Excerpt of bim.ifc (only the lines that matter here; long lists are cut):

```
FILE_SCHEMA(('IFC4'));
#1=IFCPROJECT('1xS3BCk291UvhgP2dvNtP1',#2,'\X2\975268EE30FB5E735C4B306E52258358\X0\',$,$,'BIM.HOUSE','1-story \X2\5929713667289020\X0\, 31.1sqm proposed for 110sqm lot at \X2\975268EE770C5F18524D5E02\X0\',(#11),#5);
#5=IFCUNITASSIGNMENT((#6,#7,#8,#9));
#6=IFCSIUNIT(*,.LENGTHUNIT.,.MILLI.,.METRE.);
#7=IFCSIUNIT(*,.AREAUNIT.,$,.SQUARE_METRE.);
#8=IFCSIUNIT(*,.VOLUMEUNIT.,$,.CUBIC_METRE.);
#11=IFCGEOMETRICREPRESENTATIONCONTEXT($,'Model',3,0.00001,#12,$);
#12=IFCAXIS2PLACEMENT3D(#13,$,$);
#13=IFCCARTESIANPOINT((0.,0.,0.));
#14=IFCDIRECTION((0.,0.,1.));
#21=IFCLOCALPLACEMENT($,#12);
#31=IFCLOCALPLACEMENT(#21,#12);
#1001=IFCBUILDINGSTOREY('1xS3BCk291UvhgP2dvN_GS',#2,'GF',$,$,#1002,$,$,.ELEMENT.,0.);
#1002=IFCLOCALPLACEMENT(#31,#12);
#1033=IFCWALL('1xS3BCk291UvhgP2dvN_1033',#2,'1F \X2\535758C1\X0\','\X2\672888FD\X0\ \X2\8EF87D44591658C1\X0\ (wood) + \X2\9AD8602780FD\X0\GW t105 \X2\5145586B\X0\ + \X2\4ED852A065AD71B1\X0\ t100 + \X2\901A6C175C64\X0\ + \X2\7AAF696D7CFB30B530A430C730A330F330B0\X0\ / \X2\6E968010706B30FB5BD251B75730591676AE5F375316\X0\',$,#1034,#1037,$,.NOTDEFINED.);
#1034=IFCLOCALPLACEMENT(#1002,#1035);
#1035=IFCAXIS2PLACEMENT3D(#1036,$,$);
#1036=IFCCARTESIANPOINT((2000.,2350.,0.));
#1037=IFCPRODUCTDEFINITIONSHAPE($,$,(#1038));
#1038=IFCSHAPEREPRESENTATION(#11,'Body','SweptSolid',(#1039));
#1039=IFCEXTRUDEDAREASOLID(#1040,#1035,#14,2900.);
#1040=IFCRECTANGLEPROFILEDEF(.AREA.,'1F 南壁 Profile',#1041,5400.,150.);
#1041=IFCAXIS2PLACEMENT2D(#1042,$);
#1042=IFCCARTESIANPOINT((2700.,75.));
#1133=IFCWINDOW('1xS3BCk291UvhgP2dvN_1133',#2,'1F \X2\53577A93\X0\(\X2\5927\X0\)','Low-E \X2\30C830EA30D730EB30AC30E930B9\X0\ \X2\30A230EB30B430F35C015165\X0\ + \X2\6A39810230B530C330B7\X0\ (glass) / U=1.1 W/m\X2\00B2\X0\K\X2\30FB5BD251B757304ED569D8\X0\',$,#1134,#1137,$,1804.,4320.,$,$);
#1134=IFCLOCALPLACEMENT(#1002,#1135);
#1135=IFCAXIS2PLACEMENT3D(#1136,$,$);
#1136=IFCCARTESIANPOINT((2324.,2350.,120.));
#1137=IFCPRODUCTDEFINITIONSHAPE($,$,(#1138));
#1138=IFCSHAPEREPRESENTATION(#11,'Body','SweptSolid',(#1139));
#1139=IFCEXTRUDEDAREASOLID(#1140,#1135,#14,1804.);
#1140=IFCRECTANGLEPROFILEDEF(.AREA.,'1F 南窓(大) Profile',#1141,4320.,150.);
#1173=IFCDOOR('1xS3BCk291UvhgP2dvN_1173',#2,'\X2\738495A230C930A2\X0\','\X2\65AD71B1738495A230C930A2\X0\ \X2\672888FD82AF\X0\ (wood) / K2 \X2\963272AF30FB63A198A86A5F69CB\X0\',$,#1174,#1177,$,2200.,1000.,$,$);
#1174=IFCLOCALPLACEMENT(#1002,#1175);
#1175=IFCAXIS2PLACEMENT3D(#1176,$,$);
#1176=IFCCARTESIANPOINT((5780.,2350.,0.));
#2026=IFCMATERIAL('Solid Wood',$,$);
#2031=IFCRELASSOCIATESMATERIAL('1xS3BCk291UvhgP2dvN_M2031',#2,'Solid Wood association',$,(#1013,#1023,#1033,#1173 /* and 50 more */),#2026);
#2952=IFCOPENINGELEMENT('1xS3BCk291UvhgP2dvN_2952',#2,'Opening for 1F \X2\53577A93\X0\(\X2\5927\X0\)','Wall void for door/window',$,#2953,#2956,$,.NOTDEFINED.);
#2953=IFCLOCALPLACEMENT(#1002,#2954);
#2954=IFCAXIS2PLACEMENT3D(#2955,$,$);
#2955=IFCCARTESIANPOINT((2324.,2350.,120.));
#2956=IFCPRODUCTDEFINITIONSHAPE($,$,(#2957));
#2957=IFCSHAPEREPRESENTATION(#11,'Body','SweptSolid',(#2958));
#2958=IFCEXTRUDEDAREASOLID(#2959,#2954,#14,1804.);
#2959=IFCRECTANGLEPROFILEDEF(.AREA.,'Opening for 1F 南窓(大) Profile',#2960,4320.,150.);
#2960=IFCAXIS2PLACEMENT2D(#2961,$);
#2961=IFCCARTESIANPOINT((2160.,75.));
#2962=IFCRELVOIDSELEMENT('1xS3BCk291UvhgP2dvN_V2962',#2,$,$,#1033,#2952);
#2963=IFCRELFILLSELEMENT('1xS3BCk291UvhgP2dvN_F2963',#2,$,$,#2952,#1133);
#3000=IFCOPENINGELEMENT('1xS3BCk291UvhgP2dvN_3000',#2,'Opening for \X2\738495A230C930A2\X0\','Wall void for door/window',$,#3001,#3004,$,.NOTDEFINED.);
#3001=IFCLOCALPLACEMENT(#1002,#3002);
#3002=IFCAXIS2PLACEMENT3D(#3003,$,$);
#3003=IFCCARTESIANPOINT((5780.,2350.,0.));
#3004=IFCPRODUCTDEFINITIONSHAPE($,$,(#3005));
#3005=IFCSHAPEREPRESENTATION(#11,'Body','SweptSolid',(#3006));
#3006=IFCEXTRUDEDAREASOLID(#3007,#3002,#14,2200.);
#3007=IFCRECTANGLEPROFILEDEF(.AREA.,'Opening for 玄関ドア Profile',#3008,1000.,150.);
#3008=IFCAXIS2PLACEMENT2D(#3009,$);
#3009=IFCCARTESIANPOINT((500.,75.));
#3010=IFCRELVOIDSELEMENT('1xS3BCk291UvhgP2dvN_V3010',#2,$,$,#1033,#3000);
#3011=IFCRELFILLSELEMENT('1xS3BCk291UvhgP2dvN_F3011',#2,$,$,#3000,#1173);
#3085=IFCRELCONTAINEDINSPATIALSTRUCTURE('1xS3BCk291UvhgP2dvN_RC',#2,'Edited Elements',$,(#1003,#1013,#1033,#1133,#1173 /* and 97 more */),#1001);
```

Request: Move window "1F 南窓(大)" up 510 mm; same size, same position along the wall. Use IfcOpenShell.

```python
import numpy as np
import ifcopenshell
import ifcopenshell.api.geometry
import ifcopenshell.util.placement
import ifcopenshell.util.unit

model = ifcopenshell.open("bim.ifc")
unit_scale = ifcopenshell.util.unit.calculate_unit_scale(model)

window = model.by_guid("1xS3BCk291UvhgP2dvN_1133")
opening = window.FillsVoids[0].RelatingOpeningElement
dz = 0.51 / unit_scale

shift = np.array([0.0, 0.0, dz])
# The window is not placed relative to its opening, so move both.
for product in (opening, window):
    matrix = ifcopenshell.util.placement.get_local_placement(product.ObjectPlacement)
    matrix[:3, 3] += shift
    ifcopenshell.api.geometry.edit_object_placement(model, product=product, matrix=matrix, is_si=False)

print(f"moved by {dz * unit_scale:+.3f} m")

model.write("bim_edited.ifc")
```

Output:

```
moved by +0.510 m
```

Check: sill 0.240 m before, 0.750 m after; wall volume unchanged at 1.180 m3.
